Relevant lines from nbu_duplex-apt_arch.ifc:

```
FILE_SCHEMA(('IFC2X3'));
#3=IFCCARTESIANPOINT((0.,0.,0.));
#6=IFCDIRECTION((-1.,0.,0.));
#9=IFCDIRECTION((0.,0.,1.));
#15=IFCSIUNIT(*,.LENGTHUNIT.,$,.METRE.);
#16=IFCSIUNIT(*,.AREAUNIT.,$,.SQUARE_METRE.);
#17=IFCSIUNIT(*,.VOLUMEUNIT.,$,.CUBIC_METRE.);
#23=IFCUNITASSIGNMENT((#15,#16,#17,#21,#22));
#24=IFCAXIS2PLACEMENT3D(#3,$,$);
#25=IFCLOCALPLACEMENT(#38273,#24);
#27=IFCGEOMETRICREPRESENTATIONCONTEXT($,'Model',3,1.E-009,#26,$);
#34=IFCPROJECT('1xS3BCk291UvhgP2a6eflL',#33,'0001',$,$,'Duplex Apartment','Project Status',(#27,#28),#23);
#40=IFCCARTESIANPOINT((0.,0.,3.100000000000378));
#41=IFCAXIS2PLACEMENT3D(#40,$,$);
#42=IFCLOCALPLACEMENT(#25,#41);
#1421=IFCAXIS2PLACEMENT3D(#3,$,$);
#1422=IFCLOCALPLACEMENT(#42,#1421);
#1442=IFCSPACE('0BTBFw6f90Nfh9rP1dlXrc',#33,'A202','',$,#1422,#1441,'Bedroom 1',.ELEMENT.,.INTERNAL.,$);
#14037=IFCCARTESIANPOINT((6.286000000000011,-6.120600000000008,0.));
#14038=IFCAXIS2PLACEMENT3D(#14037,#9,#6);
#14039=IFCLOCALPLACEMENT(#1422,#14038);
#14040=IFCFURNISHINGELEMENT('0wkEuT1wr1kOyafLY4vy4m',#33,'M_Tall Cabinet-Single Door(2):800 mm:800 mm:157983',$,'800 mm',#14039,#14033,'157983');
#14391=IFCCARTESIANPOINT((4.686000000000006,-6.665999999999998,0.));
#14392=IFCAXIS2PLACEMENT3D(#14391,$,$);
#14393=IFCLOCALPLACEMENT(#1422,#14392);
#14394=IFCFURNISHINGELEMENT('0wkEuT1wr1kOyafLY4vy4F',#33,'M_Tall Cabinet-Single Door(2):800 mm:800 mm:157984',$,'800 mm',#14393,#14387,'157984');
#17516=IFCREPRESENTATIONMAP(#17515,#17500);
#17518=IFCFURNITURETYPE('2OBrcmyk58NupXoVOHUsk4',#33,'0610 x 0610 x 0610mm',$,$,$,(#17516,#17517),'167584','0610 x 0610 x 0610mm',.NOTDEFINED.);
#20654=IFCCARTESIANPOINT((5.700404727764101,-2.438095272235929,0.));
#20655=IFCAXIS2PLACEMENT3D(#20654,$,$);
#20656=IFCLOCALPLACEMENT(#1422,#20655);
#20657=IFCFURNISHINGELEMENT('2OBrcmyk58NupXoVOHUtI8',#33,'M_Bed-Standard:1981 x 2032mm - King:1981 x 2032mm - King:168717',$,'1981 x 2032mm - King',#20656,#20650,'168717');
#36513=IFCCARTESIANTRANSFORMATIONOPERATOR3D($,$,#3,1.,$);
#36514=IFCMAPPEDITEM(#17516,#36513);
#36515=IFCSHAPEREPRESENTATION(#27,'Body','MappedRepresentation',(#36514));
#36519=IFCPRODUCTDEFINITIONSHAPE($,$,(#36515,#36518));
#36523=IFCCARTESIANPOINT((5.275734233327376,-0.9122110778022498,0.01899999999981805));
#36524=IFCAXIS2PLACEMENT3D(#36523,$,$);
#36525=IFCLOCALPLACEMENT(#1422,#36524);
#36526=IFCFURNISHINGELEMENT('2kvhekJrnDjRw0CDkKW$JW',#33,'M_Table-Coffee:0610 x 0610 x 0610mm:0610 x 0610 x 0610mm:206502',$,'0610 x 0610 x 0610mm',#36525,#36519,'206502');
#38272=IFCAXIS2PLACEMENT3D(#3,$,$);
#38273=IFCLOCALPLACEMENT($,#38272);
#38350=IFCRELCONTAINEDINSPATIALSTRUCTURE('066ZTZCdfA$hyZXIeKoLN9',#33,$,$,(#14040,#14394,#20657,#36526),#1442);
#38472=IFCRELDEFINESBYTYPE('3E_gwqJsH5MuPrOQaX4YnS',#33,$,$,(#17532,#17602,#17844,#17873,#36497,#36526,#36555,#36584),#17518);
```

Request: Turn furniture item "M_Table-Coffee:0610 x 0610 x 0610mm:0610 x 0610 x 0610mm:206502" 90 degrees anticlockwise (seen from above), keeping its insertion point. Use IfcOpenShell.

```python
import ifcopenshell
import ifcopenshell.api.geometry
import ifcopenshell.util.placement

model = ifcopenshell.open("nbu_duplex-apt_arch.ifc")

item = model.by_guid("2kvhekJrnDjRw0CDkKW$JW")
matrix = ifcopenshell.util.placement.get_local_placement(item.ObjectPlacement)
matrix = matrix @ ifcopenshell.util.placement.rotation(90, "Z")
ifcopenshell.api.geometry.edit_object_placement(model, product=item, matrix=matrix, is_si=False)

print(ifcopenshell.util.placement.get_local_placement(item.ObjectPlacement).round(3) + 0.0)

model.write("nbu_duplex-apt_arch_edited.ifc")
```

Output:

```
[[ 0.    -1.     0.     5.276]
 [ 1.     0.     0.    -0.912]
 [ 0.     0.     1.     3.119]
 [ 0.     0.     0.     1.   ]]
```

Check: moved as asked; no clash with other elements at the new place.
